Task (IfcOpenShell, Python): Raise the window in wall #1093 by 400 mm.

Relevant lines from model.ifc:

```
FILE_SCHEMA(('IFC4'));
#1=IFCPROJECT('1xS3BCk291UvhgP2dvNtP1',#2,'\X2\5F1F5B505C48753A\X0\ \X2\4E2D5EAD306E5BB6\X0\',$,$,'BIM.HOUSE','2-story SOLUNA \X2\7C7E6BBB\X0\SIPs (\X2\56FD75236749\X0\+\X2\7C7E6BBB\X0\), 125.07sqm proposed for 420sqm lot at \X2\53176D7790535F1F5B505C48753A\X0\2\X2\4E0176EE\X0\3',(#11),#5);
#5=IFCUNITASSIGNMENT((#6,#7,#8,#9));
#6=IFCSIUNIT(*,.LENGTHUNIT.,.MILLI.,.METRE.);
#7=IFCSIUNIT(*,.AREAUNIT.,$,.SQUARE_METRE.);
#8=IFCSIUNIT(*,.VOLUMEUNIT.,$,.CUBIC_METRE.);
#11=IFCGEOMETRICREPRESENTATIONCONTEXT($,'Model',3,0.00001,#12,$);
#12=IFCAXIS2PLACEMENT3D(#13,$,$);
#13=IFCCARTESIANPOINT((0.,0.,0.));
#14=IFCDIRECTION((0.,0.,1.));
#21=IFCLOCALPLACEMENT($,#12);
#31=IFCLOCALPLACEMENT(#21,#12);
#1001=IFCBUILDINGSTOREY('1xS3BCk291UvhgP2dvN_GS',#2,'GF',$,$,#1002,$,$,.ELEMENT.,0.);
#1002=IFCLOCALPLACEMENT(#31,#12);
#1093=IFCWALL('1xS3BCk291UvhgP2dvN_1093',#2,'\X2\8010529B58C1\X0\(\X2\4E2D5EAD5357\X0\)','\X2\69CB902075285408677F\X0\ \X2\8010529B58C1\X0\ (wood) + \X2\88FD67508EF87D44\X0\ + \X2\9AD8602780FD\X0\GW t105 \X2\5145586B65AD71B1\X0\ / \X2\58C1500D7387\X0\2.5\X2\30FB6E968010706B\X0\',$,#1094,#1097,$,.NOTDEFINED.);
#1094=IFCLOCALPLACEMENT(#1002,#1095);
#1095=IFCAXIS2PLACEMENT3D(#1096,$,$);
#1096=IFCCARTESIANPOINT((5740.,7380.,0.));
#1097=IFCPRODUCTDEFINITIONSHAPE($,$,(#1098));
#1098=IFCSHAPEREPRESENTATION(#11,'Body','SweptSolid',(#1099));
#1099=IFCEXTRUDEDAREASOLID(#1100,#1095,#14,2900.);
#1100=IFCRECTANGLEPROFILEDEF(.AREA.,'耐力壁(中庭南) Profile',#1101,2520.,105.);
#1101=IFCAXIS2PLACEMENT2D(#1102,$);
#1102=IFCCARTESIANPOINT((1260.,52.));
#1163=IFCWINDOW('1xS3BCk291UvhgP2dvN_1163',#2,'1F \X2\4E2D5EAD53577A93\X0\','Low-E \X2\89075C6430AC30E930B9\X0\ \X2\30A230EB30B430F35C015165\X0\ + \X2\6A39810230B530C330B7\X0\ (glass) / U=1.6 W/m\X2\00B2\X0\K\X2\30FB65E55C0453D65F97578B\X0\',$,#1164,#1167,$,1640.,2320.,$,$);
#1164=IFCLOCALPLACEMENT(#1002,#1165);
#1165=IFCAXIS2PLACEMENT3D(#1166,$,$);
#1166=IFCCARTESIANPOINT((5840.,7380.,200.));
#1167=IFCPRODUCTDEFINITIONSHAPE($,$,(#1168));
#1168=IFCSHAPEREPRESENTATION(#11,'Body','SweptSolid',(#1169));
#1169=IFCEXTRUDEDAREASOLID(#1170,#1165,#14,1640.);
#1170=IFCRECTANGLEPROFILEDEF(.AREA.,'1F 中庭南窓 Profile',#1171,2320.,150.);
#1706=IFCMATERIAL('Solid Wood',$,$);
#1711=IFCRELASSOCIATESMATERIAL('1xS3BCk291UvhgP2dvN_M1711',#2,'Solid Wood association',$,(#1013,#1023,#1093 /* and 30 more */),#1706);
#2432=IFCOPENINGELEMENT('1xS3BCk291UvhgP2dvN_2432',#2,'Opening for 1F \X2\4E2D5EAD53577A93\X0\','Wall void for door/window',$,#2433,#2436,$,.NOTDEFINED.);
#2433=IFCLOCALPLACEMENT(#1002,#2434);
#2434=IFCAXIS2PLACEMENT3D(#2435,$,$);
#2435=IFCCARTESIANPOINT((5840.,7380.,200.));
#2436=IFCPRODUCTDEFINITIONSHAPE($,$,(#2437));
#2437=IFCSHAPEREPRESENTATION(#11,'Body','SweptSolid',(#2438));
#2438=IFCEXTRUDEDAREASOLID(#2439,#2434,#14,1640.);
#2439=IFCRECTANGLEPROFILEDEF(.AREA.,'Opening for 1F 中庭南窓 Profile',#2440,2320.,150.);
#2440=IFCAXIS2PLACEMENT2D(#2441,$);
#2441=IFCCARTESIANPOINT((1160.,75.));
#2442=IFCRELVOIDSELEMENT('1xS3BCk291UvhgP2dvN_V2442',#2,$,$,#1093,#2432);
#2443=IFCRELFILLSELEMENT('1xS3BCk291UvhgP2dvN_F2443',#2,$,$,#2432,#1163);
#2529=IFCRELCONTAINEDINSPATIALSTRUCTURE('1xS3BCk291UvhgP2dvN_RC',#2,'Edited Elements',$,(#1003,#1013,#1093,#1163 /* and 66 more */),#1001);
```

```python
import numpy as np
import ifcopenshell
import ifcopenshell.api.geometry
import ifcopenshell.util.placement
import ifcopenshell.util.unit

model = ifcopenshell.open("model.ifc")
unit_scale = ifcopenshell.util.unit.calculate_unit_scale(model)

window = model.by_guid("1xS3BCk291UvhgP2dvN_1163")
opening = window.FillsVoids[0].RelatingOpeningElement
dz = 0.4 / unit_scale

shift = np.array([0.0, 0.0, dz])
# The window is not placed relative to its opening, so move both.
for product in (opening, window):
    matrix = ifcopenshell.util.placement.get_local_placement(product.ObjectPlacement)
    matrix[:3, 3] += shift
    ifcopenshell.api.geometry.edit_object_placement(model, product=product, matrix=matrix, is_si=False)

print(f"moved by {dz * unit_scale:+.3f} m")

model.write("model_v2.ifc")
```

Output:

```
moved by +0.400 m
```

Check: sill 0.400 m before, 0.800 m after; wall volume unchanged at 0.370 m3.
